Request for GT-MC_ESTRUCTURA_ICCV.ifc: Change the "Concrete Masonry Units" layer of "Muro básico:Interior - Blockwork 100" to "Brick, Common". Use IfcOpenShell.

First a look at what the model holds.

```python
import ifcopenshell
import ifcopenshell.util.element

model = ifcopenshell.open("GT-MC_ESTRUCTURA_ICCV.ifc")
print(model.schema)
for layer_set in model.by_type("IfcMaterialLayerSet"):
    if layer_set.LayerSetName == "Muro básico:Interior - Blockwork 100":
        for layer in layer_set.MaterialLayers:
            print(layer.id(), layer.Material and layer.Material.Name, layer.LayerThickness, sep=" | ")
        print(len(ifcopenshell.util.element.get_elements_by_material(model, layer_set)), "elements and types use it")
print(sorted(m.Name for m in model.by_type("IfcMaterial") if m.Name)[:60])
```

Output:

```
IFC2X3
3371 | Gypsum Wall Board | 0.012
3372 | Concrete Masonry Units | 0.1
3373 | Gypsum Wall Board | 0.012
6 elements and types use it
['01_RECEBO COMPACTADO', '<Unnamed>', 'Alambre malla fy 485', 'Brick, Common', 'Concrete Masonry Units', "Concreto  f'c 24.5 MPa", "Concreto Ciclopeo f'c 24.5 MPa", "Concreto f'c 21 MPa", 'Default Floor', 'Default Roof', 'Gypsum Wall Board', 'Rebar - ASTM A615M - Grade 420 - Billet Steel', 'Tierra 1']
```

```python
import ifcopenshell
import ifcopenshell.api.material

model = ifcopenshell.open("GT-MC_ESTRUCTURA_ICCV.ifc")

layer_set = next(s for s in model.by_type("IfcMaterialLayerSet") if s.LayerSetName == "Muro básico:Interior - Blockwork 100")
layer = next(l for l in layer_set.MaterialLayers if l.Material and l.Material.Name == "Concrete Masonry Units")
material = next(m for m in model.by_type("IfcMaterial") if m.Name == "Brick, Common")

# Point this one layer at the other material; renaming the old one would change it everywhere.
ifcopenshell.api.material.edit_layer(model, layer=layer, attributes={}, material=material)

print([l.Material.Name if l.Material else None for l in layer_set.MaterialLayers])

model.write("GT-MC_ESTRUCTURA_ICCV_edited.ifc")
```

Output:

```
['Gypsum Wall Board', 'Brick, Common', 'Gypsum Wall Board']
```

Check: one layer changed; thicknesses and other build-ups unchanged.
